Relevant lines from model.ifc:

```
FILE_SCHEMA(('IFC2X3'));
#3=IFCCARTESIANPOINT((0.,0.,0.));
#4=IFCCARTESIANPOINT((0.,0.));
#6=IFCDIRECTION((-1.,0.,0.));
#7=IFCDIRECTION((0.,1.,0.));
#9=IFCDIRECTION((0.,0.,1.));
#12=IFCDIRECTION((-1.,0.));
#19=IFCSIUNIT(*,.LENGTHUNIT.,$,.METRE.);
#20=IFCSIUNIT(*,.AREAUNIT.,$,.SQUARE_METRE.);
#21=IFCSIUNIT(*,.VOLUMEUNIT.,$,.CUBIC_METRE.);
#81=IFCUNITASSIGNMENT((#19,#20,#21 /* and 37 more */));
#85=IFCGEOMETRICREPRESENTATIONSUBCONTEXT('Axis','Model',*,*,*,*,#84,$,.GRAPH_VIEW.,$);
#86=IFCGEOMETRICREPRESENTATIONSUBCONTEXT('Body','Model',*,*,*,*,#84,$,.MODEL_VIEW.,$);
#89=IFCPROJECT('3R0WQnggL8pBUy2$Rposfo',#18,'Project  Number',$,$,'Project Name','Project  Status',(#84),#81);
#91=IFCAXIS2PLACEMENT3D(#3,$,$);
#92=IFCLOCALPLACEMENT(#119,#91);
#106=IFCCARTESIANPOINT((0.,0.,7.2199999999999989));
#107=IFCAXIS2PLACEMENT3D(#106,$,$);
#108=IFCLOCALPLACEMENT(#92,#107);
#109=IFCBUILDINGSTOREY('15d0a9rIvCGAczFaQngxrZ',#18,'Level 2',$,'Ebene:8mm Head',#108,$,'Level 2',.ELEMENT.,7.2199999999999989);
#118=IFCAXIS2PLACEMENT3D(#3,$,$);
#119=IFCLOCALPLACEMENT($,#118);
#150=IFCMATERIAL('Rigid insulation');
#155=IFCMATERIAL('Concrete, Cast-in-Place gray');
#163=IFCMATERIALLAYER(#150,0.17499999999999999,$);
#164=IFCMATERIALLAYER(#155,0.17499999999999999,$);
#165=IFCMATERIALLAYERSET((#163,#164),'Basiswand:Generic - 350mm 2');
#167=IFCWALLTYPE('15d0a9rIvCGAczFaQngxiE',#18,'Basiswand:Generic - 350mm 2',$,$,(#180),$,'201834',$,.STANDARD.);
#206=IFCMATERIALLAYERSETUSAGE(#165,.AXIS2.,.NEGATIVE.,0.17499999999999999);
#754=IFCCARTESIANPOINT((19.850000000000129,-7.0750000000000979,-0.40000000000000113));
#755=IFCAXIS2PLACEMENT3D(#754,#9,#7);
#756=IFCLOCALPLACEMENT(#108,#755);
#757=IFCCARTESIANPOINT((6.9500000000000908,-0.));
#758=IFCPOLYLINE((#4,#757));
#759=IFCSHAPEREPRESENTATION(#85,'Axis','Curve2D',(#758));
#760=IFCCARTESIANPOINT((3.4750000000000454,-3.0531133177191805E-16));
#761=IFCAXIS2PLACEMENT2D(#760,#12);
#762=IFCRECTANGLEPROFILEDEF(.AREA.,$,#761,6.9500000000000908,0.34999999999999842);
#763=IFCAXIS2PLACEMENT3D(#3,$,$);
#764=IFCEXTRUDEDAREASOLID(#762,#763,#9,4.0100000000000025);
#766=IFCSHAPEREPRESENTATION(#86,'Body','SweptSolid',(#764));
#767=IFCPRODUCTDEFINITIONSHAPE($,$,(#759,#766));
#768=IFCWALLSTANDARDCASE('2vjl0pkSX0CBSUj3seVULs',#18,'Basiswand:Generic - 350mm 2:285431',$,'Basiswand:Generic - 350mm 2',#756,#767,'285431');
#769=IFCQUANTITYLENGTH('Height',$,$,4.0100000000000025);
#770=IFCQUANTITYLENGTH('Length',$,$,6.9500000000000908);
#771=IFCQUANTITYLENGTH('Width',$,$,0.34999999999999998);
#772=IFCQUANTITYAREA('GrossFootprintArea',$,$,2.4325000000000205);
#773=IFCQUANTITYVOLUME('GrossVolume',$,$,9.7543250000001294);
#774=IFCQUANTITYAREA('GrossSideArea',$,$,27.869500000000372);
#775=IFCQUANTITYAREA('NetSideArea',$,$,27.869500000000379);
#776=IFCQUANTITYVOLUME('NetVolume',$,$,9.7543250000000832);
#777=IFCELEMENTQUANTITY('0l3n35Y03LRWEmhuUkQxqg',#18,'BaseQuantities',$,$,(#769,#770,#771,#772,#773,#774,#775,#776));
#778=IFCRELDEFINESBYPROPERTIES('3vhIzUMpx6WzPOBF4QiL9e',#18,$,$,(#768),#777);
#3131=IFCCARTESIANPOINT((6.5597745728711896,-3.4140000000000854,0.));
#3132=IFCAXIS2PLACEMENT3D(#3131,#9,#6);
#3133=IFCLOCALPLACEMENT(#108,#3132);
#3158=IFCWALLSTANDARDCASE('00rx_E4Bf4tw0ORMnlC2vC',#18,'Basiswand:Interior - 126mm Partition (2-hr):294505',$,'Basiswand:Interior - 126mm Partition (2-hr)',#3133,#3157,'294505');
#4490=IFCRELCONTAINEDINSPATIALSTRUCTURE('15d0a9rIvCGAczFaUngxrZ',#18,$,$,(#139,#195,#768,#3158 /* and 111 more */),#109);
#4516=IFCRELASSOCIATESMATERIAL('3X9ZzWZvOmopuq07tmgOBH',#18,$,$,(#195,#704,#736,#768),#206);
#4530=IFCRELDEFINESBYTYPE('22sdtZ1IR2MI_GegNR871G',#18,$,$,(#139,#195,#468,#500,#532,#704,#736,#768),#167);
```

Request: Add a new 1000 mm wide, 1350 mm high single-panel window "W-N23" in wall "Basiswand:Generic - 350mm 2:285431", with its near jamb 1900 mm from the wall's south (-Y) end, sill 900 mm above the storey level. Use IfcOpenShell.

```python
import numpy as np
import ifcopenshell
import ifcopenshell.api.feature
import ifcopenshell.api.geometry
import ifcopenshell.api.pset
import ifcopenshell.api.root
import ifcopenshell.api.spatial
import ifcopenshell.api.type
import ifcopenshell.geom
import ifcopenshell.util.element
import ifcopenshell.util.placement
import ifcopenshell.util.representation
import ifcopenshell.util.shape
import ifcopenshell.util.unit

model = ifcopenshell.open("model.ifc")
unit_scale = ifcopenshell.util.unit.calculate_unit_scale(model)
area_scale = ifcopenshell.util.unit.calculate_unit_scale(model, "AREAUNIT")
volume_scale = ifcopenshell.util.unit.calculate_unit_scale(model, "VOLUMEUNIT")
settings = ifcopenshell.geom.settings()


def volume(element):
    """Net volume in cubic metres, openings subtracted."""
    shape = ifcopenshell.geom.create_shape(settings, element)
    return ifcopenshell.util.shape.get_volume(shape.geometry)


wall = model.by_id(768)
storey = ifcopenshell.util.element.get_container(wall, ifc_class="IfcBuildingStorey")
context = ifcopenshell.util.representation.get_context(model, "Model", "Body", "MODEL_VIEW")
before = volume(wall)

width, height, from_end, sill = 1, 1.35, 1.9, 0.9  # metres

# The wall runs along its own X axis, and the end named is its -X end.
wall_shape = ifcopenshell.geom.create_shape(settings, wall)
x, y, z = ifcopenshell.util.shape.get_vertices(wall_shape.geometry).T
start = x.min() + from_end
face, thickness = float(y.min()), float(y.max() - y.min())
wall_matrix = ifcopenshell.util.placement.get_local_placement(wall.ObjectPlacement)
level = ifcopenshell.util.placement.get_local_placement(storey.ObjectPlacement)[2, 3]


def in_wall(x, y):
    """Placement at x, y metres in the wall's axes, at sill height."""
    matrix = wall_matrix.copy()
    matrix[:, 3] = wall_matrix @ np.array([x / unit_scale, y / unit_scale, 0.0, 1.0])
    matrix[2, 3] = level + sill / unit_scale
    return matrix


# Opening: a box that overshoots both wall faces by 50 mm.
opening = ifcopenshell.api.root.create_entity(model, ifc_class="IfcOpeningElement")
box = ifcopenshell.api.geometry.add_wall_representation(
    model, context=context, length=width, height=height, thickness=thickness + 0.1
)
ifcopenshell.api.geometry.assign_representation(model, product=opening, representation=box)
ifcopenshell.api.geometry.edit_object_placement(model, product=opening, matrix=in_wall(start, face - 0.05), is_si=False)
ifcopenshell.api.feature.add_feature(model, feature=opening, element=wall)

window = ifcopenshell.api.root.create_entity(model, ifc_class="IfcWindow", name="W-N23")
window.OverallWidth, window.OverallHeight = width / unit_scale, height / unit_scale
body = ifcopenshell.api.geometry.add_window_representation(
    model,
    context=context,
    overall_width=window.OverallWidth,
    overall_height=window.OverallHeight,
    partition_type="SINGLE_PANEL",
)
ifcopenshell.api.geometry.assign_representation(model, product=window, representation=body)
ifcopenshell.api.spatial.assign_container(model, products=[window], relating_structure=storey)
fills = ifcopenshell.api.feature.add_filling(model, opening=opening, element=window)
fills.OwnerHistory = window.OwnerHistory  # required in IFC2X3

# IFC2X3 keeps the operation on the window style.
style = ifcopenshell.api.root.create_entity(model, ifc_class="IfcWindowStyle", name="W-N23")
style.OperationType, style.ConstructionType = "SINGLE_PANEL", "NOTDEFINED"
style.ParameterTakesPrecedence = style.Sizeable = False
ifcopenshell.api.type.assign_type(model, related_objects=[window], relating_type=style)

# Centre the window in the wall's thickness.
ifcopenshell.api.geometry.edit_object_placement(model, product=window, matrix=in_wall(start, face), is_si=False)
window_shape = ifcopenshell.geom.create_shape(settings, window)
depth = ifcopenshell.util.shape.get_vertices(window_shape.geometry)[:, 1]
offset = face + thickness / 2 - (depth.min() + depth.max()) / 2
ifcopenshell.api.geometry.edit_object_placement(model, product=window, matrix=in_wall(start, offset), is_si=False)

after = volume(wall)

# Update the wall's stored quantities.
qto = model.by_id(ifcopenshell.util.element.get_pset(wall, "BaseQuantities", should_inherit=False)["id"])
ifcopenshell.api.pset.edit_qto(model, qto=qto, properties={
    "NetSideArea": after / thickness / area_scale,
    "NetVolume": after / volume_scale,
})

print(f"wall volume {before:.3f} -> {after:.3f} m3")

model.write("model_rev.ifc")
```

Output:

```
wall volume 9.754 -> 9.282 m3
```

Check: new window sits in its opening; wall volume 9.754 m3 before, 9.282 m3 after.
